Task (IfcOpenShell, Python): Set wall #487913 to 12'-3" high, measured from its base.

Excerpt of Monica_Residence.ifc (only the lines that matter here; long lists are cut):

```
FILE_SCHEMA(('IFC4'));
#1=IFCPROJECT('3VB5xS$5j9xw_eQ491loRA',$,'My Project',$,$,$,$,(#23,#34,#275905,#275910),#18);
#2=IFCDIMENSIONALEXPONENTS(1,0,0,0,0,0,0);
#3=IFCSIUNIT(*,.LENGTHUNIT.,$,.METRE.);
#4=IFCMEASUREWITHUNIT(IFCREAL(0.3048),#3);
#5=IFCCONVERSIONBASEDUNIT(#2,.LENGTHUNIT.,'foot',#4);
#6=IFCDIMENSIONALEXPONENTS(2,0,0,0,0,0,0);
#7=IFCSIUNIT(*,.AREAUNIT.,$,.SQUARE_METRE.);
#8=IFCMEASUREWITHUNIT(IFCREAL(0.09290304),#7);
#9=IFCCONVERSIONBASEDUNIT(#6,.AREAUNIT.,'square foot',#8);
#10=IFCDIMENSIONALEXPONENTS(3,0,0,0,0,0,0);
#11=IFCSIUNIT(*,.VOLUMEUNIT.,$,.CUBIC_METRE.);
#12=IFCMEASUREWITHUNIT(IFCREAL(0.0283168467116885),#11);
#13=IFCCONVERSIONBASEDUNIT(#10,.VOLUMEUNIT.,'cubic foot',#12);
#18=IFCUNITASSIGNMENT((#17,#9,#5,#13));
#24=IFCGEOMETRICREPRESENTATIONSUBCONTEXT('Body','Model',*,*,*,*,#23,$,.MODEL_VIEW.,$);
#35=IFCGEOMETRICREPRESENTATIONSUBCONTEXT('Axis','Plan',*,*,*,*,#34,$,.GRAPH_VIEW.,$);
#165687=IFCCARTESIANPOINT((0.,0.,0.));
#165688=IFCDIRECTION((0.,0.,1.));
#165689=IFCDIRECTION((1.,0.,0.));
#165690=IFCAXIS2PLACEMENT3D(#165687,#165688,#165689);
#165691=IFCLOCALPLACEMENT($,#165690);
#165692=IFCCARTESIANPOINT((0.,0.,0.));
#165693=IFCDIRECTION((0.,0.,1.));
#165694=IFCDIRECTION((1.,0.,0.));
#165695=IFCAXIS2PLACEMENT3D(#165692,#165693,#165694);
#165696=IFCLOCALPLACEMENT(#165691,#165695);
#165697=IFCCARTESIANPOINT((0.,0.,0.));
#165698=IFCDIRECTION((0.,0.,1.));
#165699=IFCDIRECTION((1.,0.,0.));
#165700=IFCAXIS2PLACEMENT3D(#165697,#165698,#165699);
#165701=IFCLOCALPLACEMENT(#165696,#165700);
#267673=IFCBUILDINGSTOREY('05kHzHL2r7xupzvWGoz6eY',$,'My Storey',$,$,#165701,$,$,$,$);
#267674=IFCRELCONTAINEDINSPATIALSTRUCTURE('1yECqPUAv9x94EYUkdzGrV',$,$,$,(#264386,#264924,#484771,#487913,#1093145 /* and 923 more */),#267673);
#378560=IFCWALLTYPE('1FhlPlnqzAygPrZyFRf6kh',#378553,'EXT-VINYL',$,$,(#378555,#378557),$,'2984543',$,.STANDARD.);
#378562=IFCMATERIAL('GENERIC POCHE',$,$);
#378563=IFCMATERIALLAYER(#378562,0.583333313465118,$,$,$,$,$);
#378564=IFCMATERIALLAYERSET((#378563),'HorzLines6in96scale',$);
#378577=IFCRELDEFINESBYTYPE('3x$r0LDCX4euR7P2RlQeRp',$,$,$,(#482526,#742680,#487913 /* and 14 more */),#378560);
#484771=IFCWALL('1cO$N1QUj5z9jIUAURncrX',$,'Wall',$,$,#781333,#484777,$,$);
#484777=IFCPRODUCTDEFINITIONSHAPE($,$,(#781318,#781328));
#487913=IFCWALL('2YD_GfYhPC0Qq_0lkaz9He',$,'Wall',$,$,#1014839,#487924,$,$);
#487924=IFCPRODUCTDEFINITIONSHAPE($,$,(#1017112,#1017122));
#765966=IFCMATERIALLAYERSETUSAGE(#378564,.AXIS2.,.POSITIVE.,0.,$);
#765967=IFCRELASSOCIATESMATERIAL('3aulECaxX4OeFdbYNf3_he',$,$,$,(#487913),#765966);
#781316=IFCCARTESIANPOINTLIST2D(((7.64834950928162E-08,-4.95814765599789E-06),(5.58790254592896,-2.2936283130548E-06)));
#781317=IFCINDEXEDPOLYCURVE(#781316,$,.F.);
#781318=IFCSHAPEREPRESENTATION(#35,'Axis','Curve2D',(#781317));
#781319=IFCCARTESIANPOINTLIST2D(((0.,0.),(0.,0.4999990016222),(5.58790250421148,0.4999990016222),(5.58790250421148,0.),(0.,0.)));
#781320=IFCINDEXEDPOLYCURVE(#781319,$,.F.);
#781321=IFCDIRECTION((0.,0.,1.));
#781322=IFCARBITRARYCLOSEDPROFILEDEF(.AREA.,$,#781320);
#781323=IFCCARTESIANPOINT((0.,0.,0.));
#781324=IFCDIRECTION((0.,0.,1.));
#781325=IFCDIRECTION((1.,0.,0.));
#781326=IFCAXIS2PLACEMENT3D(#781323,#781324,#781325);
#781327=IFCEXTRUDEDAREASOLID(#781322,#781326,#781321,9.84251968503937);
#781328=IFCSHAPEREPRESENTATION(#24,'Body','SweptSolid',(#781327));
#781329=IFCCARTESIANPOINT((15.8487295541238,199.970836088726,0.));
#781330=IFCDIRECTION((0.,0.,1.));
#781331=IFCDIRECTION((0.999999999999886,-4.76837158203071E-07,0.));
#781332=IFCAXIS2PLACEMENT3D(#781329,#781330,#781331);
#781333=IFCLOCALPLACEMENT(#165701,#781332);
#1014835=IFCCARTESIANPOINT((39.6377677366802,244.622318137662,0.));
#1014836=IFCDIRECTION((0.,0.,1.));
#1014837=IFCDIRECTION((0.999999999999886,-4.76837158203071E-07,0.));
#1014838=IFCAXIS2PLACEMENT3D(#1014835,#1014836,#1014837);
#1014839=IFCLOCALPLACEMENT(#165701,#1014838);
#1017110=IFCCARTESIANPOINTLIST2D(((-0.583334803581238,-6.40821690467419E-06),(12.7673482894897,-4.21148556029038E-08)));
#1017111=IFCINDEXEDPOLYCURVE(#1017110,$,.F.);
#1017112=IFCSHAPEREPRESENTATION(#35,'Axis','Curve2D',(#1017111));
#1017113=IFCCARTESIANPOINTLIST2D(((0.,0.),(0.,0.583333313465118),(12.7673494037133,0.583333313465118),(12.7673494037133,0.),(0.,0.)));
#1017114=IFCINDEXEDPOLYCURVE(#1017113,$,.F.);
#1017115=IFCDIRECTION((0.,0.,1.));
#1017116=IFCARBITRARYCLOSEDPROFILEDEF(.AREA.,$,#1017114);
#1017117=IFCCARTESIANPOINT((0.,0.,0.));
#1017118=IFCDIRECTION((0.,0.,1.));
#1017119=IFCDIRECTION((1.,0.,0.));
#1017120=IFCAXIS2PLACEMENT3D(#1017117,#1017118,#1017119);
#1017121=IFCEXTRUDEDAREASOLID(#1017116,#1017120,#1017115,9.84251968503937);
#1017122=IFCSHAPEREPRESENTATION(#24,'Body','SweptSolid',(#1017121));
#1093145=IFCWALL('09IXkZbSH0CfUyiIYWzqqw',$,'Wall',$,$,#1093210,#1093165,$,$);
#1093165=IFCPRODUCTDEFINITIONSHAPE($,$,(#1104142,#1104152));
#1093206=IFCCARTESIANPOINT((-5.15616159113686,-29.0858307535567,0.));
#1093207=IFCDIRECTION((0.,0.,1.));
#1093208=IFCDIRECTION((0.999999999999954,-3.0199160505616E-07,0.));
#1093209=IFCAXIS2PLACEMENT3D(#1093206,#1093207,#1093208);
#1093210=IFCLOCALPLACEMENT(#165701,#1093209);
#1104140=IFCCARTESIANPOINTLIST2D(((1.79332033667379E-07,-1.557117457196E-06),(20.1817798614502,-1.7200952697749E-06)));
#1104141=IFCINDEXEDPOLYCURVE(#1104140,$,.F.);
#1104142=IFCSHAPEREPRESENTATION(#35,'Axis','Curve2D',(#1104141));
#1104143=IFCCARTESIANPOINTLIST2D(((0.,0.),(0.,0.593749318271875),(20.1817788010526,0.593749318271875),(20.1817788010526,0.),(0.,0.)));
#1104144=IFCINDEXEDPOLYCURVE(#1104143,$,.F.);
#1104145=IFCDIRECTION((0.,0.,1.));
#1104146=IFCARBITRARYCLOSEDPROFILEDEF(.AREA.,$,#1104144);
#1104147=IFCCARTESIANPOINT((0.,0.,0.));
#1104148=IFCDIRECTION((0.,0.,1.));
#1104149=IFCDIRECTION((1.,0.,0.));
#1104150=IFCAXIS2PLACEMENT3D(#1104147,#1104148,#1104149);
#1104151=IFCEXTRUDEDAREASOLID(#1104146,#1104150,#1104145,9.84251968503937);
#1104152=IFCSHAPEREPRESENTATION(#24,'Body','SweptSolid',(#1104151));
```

```python
import ifcopenshell
import ifcopenshell.geom
import ifcopenshell.util.representation
import ifcopenshell.util.shape
import ifcopenshell.util.unit

model = ifcopenshell.open("Monica_Residence.ifc")
unit_scale = ifcopenshell.util.unit.calculate_unit_scale(model)
settings = ifcopenshell.geom.settings()


def volume(element):
    """Net volume in cubic metres, openings subtracted."""
    shape = ifcopenshell.geom.create_shape(settings, element)
    return ifcopenshell.util.shape.get_volume(shape.geometry)


wall = model.by_guid("2YD_GfYhPC0Qq_0lkaz9He")
before = volume(wall)

body = ifcopenshell.util.representation.get_representation(wall, "Model", "Body")
solid = body.Items[0]
old_height = solid.Depth
solid.Depth = 147 * 0.0254 / unit_scale
after = volume(wall)

print(f"height {old_height:g} -> {solid.Depth:g}, volume {before:.3f} -> {after:.3f} m3")

model.write("Monica_Residence_edited.ifc")
```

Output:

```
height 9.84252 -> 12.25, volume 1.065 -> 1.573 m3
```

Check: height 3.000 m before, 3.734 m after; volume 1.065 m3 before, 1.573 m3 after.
